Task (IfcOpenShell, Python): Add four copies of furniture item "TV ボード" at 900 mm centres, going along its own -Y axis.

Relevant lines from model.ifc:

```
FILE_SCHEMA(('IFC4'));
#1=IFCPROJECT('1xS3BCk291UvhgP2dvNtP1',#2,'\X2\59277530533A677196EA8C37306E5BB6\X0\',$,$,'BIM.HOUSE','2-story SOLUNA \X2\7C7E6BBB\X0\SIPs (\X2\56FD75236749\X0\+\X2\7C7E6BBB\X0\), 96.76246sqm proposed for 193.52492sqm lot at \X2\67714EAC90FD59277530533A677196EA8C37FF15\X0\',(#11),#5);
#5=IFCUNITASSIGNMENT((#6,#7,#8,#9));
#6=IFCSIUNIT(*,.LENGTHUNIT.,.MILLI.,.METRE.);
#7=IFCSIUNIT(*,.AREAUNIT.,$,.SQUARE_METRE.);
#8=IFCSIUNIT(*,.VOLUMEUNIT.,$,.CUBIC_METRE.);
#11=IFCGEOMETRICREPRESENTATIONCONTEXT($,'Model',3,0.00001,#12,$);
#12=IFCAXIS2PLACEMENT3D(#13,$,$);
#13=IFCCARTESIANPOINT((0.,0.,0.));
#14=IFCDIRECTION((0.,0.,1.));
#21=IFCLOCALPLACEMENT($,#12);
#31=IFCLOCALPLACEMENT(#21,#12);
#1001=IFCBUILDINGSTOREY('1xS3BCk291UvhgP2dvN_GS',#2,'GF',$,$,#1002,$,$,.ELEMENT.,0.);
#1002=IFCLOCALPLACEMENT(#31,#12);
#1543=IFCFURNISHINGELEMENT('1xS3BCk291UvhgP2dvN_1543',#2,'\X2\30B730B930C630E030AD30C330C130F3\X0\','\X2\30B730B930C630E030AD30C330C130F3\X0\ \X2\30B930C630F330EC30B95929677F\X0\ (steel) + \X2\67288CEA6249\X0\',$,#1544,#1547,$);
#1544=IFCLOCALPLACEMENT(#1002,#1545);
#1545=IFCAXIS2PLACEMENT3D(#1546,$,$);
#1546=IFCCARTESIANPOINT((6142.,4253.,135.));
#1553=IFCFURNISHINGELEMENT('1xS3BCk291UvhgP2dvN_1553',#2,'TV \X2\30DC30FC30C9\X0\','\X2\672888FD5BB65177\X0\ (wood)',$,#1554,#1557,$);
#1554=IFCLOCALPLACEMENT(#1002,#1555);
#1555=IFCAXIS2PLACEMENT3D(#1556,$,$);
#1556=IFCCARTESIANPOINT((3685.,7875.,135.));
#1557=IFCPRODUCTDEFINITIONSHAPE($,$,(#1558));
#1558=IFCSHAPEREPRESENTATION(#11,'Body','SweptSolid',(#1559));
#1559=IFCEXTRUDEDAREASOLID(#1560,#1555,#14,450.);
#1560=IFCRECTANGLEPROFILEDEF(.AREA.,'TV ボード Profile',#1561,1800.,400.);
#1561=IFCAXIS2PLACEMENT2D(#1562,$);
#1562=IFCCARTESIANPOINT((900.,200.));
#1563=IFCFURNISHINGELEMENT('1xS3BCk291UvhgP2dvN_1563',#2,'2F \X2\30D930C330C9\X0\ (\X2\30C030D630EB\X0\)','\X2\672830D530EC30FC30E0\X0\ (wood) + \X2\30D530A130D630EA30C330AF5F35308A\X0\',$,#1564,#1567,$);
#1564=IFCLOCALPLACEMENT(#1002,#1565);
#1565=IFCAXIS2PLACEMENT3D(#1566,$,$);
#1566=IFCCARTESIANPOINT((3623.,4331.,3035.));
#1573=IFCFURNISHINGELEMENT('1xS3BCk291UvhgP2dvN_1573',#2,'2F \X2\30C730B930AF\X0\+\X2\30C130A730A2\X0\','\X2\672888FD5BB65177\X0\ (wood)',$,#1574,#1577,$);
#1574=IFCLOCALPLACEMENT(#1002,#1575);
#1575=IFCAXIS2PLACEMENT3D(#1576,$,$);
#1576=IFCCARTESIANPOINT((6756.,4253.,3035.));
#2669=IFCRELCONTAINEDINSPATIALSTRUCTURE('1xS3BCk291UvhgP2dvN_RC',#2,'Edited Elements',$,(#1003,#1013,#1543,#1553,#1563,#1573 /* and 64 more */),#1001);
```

```python
import ifcopenshell
import ifcopenshell.api.geometry
import ifcopenshell.api.root
import ifcopenshell.util.element
import ifcopenshell.util.placement
import ifcopenshell.util.unit

model = ifcopenshell.open("model.ifc")
unit_scale = ifcopenshell.util.unit.calculate_unit_scale(model)


def reuse_history(source, copy):
    """copy_class also copies each property set's owner history, people and application; keep the originals."""
    for rel in copy.IsDefinedBy:
        if rel.is_a("IfcRelDefinesByProperties") and (history := rel.RelatingPropertyDefinition.OwnerHistory):
            rel.RelatingPropertyDefinition.OwnerHistory = source.OwnerHistory
            ifcopenshell.util.element.remove_deep2(model, history)


source = model.by_guid("1xS3BCk291UvhgP2dvN_1553")
base = ifcopenshell.util.placement.get_local_placement(source.ObjectPlacement)
step = -base[:3, 1] * 0.9 / unit_scale

for i in range(1, 5):
    copy = ifcopenshell.api.root.copy_class(model, product=source)
    copy.Representation = ifcopenshell.util.element.copy_deep(
        model, source.Representation, exclude=["IfcGeometricRepresentationContext", "IfcRepresentationMap"]
    )
    reuse_history(source, copy)
    matrix = base.copy()
    matrix[:3, 3] += i * step
    print("added at", matrix[:3, 3].round(3) + 0.0)
    ifcopenshell.api.geometry.edit_object_placement(model, product=copy, matrix=matrix, is_si=False)

model.write("model_edited.ifc")
```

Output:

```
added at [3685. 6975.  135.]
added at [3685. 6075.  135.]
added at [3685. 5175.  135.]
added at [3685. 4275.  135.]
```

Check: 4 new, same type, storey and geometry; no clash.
